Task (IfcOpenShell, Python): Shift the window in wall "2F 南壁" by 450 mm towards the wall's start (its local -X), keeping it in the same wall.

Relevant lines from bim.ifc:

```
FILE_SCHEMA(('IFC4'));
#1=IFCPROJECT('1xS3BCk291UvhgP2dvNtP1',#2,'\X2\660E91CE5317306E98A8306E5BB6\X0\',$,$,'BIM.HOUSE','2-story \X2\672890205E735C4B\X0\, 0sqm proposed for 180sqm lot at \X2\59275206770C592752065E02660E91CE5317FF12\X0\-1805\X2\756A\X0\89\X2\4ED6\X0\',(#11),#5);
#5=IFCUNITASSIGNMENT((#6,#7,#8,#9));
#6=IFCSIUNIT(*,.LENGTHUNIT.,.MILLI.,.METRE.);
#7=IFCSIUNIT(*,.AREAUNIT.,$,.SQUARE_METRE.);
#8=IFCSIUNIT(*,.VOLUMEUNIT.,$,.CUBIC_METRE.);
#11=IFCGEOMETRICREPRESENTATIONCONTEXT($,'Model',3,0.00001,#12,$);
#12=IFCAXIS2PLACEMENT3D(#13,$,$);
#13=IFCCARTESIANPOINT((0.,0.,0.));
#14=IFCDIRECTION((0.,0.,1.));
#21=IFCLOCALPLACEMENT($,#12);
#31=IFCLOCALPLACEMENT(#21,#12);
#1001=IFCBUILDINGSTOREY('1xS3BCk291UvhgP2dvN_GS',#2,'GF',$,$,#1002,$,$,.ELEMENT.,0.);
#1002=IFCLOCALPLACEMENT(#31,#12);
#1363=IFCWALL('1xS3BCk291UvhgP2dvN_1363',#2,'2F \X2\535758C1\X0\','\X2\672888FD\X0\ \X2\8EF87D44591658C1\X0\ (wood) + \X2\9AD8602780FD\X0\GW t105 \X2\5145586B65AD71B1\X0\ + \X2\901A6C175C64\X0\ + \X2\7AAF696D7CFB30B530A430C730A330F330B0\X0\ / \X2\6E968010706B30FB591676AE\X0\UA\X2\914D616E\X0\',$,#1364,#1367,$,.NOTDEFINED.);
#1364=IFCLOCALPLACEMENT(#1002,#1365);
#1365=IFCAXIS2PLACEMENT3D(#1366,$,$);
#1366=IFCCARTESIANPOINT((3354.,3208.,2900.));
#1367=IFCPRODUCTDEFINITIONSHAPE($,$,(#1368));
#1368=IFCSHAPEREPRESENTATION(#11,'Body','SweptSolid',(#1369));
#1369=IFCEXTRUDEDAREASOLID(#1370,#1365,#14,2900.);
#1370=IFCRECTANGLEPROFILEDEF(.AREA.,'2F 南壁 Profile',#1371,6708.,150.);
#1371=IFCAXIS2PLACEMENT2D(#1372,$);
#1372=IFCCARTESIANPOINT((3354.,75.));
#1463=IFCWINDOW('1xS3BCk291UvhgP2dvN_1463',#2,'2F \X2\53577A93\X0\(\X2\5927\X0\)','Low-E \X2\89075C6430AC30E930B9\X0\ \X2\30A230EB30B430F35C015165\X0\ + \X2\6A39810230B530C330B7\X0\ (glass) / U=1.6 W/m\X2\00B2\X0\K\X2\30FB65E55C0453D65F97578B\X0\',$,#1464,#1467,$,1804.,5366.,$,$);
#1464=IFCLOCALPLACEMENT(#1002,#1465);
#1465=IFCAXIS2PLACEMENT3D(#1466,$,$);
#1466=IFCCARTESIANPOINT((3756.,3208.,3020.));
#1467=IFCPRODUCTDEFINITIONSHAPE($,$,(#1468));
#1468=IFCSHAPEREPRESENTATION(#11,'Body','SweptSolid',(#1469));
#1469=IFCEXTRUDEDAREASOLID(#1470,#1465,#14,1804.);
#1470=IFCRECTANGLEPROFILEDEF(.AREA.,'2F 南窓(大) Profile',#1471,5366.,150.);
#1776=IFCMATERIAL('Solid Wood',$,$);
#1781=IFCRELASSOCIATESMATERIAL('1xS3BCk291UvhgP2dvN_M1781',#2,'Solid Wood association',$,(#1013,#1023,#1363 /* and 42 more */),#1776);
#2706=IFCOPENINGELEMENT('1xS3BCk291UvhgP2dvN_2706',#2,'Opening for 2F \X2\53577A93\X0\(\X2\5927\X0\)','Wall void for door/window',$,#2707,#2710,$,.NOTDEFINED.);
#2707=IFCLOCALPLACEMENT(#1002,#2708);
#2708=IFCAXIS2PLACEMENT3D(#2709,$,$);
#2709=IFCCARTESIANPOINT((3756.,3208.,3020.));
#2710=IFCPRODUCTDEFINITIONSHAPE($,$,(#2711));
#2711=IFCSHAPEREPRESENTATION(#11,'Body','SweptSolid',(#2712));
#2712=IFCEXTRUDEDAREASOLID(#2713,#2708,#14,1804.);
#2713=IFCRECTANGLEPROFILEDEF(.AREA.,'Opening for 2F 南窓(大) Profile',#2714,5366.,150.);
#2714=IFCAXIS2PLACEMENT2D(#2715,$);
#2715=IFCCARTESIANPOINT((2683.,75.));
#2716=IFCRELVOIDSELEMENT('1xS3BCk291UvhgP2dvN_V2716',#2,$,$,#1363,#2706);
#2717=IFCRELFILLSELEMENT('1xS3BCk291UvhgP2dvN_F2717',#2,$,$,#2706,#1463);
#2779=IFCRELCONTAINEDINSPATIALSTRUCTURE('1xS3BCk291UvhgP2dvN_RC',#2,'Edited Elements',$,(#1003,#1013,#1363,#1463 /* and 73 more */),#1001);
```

```python
import ifcopenshell
import ifcopenshell.api.geometry
import ifcopenshell.util.placement

model = ifcopenshell.open("bim.ifc")

window = model.by_guid("1xS3BCk291UvhgP2dvN_1463")
opening = window.FillsVoids[0].RelatingOpeningElement
wall = opening.VoidsElements[0].RelatingBuildingElement

wall_matrix = ifcopenshell.util.placement.get_local_placement(wall.ObjectPlacement)
shift = wall_matrix[:3, 0] * -450.0
before = ifcopenshell.util.placement.get_local_placement(window.ObjectPlacement)[:3, 3].copy()

# The window is not placed relative to its opening, so move both.
for product in (opening, window):
    matrix = ifcopenshell.util.placement.get_local_placement(product.ObjectPlacement)
    matrix[:3, 3] += shift
    ifcopenshell.api.geometry.edit_object_placement(model, product=product, matrix=matrix, is_si=False)

after = ifcopenshell.util.placement.get_local_placement(window.ObjectPlacement)[:3, 3]
print("window moved by", (after - before).round(3) + 0.0)

model.write("bim_rev.ifc")
```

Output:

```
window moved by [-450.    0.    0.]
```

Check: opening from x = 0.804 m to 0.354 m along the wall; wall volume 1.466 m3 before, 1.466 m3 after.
